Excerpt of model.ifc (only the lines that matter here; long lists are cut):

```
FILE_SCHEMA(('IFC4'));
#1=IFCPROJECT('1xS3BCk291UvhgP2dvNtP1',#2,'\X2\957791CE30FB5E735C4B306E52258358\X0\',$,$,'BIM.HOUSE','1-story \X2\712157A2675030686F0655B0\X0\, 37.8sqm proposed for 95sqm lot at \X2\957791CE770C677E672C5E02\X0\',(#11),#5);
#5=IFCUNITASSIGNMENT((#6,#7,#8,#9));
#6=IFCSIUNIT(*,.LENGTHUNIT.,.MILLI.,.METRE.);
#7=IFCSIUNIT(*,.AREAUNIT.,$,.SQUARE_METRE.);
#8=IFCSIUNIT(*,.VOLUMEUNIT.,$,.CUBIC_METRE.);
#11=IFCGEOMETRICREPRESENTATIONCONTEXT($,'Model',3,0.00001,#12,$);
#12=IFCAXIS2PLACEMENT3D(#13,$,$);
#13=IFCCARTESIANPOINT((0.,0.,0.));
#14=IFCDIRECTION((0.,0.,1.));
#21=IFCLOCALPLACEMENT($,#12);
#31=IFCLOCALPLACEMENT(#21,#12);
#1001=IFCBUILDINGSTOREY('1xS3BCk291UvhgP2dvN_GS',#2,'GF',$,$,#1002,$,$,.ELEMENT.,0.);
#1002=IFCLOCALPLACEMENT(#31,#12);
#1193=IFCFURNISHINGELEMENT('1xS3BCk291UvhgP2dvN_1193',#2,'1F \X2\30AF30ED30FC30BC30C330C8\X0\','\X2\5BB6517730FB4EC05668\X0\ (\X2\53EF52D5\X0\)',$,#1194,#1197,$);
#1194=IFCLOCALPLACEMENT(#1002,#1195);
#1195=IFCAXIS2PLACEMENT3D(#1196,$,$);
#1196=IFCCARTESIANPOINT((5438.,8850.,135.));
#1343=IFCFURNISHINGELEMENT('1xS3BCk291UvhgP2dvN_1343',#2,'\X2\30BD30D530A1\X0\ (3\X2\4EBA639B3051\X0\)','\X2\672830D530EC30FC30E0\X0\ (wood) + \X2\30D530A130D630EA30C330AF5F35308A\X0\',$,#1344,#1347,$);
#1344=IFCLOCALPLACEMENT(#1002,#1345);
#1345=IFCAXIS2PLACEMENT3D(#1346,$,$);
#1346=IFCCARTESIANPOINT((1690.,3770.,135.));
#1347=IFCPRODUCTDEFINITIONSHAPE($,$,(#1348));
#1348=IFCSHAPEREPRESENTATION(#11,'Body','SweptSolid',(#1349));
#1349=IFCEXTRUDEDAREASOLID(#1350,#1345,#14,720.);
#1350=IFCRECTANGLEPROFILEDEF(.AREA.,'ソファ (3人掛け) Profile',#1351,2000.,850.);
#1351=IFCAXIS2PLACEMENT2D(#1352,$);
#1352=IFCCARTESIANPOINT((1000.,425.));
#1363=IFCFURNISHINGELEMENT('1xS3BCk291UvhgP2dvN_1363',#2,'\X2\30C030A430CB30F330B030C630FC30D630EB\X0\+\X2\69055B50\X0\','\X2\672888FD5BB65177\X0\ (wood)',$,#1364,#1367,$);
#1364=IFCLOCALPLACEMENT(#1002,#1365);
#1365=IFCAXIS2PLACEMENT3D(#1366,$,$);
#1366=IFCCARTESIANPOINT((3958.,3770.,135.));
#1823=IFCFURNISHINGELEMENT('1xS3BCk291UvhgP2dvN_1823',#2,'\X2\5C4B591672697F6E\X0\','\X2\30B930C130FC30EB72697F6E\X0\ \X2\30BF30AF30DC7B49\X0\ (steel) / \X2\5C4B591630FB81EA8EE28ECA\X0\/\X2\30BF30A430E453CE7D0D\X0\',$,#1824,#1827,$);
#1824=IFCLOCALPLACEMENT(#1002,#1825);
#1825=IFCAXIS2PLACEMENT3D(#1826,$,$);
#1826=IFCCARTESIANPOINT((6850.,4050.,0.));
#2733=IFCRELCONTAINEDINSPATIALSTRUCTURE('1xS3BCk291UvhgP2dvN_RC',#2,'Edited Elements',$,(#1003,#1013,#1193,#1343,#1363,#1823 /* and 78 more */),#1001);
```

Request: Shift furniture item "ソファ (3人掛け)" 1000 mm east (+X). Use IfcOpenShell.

```python
import ifcopenshell
import ifcopenshell.api.geometry
import ifcopenshell.util.placement

model = ifcopenshell.open("model.ifc")

item = model.by_guid("1xS3BCk291UvhgP2dvN_1343")
matrix = ifcopenshell.util.placement.get_local_placement(item.ObjectPlacement)
matrix[0, 3] += 1000.0
ifcopenshell.api.geometry.edit_object_placement(model, product=item, matrix=matrix, is_si=False)

print(ifcopenshell.util.placement.get_local_placement(item.ObjectPlacement).round(3) + 0.0)

model.write("model_edited.ifc")
```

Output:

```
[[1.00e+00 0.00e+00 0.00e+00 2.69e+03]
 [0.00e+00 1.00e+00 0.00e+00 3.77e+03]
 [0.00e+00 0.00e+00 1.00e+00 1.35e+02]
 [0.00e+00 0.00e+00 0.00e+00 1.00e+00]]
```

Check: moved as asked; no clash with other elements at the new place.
